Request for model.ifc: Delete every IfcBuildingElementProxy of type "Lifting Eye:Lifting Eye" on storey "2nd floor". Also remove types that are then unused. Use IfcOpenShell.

First a look at what the model holds.

```python
import ifcopenshell
import ifcopenshell.util.element

model = ifcopenshell.open("model.ifc")
print(model.schema)
storey = next(s for s in model.by_type("IfcBuildingStorey") if s.Name == "2nd floor")
proxies = [e for e in ifcopenshell.util.element.get_decomposition(storey) if e.is_a("IfcBuildingElementProxy")]
seen = {}
for e in proxies:
    element_type = ifcopenshell.util.element.get_type(e)
    name = element_type.Name if element_type not in (None, e) else None
    seen[name] = seen.get(name, 0) + 1
for name, count in sorted(seen.items(), key=str):
    print(count, "x", name)
```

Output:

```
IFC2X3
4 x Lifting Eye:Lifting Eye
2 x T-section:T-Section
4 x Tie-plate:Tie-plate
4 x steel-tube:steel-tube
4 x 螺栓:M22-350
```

```python
import ifcopenshell
import ifcopenshell.api.root
import ifcopenshell.util.element

model = ifcopenshell.open("model.ifc")

storey = next(s for s in model.by_type("IfcBuildingStorey") if s.Name == "2nd floor")
proxies = [e for e in ifcopenshell.util.element.get_decomposition(storey) if e.is_a("IfcBuildingElementProxy")]
targets = [e for e in proxies if (t := ifcopenshell.util.element.get_type(e)) not in (None, e) and t.Name == "Lifting Eye:Lifting Eye"]
types = {ifcopenshell.util.element.get_type(e) for e in targets} - {None, *targets}

for e in targets:
    ifcopenshell.api.root.remove_product(model, product=e)
print(len(targets), "removed")

unused = [t for t in types if not ifcopenshell.util.element.get_types(t)]
for t in unused:
    ifcopenshell.api.root.remove_product(model, product=t)
print(len(unused), "unused types removed")

model.write("model_updated.ifc")
```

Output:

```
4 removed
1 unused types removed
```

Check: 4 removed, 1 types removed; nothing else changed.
